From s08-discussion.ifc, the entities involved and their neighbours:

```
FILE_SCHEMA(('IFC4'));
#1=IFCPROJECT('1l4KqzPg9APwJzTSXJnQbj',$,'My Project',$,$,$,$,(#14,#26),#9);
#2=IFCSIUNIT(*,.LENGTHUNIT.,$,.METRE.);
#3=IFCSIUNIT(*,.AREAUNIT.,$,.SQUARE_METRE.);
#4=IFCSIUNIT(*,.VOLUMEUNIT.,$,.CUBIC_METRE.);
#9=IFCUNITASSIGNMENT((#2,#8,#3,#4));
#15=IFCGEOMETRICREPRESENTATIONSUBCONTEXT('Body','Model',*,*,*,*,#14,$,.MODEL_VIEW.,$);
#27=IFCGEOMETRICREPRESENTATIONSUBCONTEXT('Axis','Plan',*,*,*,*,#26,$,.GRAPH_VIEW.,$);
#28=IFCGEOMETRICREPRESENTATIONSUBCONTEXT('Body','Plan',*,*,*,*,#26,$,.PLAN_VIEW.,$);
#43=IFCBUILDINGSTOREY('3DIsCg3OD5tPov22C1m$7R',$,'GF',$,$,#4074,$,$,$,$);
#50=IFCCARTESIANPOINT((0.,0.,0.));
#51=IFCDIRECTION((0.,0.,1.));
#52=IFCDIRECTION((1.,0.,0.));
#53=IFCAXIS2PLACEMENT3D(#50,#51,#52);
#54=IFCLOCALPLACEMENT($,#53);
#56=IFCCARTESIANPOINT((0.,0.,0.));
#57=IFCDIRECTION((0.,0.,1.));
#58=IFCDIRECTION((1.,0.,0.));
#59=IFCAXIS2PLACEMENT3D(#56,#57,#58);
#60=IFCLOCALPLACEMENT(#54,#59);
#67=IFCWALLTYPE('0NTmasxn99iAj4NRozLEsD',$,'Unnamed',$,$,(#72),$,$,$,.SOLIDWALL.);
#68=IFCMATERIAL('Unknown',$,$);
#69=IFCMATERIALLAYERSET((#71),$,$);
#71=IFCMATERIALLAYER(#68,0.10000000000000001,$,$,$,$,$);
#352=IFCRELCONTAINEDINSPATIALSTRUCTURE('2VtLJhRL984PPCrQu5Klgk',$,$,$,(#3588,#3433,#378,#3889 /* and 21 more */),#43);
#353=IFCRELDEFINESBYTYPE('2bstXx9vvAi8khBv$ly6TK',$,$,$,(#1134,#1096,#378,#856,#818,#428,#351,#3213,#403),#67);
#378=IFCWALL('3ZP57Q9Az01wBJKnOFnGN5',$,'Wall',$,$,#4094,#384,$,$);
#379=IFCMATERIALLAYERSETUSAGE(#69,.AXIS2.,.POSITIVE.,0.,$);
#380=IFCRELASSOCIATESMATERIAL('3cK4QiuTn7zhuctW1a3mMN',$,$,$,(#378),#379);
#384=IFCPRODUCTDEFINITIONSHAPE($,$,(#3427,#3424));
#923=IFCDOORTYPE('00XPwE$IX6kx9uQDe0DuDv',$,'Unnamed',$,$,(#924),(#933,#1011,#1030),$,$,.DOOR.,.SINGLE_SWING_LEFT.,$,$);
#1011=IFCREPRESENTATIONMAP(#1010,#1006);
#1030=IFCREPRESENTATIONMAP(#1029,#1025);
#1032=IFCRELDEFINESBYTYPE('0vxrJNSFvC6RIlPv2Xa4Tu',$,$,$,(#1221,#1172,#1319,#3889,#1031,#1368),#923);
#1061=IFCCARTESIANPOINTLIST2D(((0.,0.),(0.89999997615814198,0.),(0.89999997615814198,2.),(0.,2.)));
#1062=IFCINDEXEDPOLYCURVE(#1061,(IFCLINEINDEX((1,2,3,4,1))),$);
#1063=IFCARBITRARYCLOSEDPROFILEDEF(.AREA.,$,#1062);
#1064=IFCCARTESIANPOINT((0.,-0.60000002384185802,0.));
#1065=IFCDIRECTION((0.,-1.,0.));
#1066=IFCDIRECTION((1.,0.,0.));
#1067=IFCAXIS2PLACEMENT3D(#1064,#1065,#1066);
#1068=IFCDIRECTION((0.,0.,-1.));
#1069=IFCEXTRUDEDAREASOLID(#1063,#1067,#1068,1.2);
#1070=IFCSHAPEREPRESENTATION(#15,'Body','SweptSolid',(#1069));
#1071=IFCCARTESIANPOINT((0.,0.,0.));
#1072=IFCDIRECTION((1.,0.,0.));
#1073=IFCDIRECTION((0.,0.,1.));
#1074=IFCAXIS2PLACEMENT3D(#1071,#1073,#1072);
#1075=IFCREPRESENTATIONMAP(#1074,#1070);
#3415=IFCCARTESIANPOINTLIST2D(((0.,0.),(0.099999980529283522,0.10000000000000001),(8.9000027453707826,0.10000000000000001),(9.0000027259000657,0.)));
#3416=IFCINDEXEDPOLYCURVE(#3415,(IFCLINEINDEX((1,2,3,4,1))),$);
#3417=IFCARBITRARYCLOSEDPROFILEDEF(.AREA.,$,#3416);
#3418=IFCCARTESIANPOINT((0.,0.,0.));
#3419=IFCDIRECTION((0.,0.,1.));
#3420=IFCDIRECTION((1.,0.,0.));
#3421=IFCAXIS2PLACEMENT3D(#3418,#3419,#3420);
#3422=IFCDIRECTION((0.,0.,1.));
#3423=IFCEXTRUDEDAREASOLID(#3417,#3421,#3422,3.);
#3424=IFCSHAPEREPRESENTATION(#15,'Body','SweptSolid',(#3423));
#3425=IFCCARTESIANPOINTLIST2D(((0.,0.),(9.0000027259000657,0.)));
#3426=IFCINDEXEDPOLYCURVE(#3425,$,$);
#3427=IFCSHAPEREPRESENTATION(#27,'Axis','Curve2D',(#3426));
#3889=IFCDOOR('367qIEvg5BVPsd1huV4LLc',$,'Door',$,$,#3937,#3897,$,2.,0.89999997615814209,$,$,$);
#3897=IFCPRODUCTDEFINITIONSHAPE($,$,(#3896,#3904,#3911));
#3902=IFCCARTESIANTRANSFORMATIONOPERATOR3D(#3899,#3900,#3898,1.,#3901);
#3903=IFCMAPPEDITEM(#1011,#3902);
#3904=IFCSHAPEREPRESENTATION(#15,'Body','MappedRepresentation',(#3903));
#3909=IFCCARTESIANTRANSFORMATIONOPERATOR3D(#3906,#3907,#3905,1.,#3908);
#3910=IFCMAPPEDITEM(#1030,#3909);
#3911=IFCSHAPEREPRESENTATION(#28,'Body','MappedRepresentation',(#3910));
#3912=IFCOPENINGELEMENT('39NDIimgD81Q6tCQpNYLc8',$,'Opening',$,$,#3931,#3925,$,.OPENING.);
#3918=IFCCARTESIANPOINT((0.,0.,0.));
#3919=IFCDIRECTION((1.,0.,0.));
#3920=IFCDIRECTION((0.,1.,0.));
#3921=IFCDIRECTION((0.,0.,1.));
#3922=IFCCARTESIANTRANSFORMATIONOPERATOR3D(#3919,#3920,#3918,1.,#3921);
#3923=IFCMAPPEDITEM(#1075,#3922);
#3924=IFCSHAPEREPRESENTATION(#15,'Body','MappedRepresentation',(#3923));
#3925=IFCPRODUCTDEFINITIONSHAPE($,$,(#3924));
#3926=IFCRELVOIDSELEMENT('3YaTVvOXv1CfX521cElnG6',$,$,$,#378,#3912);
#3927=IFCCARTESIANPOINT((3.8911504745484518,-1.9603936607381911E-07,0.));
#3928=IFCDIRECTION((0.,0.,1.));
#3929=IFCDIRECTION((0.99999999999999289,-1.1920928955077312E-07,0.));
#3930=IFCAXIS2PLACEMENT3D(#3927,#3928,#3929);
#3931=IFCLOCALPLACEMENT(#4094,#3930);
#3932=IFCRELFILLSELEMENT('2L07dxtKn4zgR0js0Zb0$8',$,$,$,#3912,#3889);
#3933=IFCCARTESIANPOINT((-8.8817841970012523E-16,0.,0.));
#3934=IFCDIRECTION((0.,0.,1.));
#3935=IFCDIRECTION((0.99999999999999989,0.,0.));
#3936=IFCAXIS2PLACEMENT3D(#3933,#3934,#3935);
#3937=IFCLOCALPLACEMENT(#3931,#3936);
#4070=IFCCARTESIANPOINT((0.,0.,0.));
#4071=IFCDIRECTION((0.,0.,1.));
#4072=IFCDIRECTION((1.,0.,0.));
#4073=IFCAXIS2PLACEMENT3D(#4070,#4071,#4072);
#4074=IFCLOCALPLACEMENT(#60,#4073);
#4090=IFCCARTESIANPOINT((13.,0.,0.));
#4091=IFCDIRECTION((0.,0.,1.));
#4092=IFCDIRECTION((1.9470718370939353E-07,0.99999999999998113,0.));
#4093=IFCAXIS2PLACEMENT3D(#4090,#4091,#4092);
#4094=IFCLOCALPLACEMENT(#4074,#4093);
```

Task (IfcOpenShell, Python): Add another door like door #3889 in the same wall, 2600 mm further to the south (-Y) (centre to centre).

```python
import ifcopenshell
import ifcopenshell.api.feature
import ifcopenshell.api.geometry
import ifcopenshell.api.root
import ifcopenshell.geom
import ifcopenshell.util.element
import ifcopenshell.util.placement
import ifcopenshell.util.shape
import ifcopenshell.util.unit

model = ifcopenshell.open("s08-discussion.ifc")
unit_scale = ifcopenshell.util.unit.calculate_unit_scale(model)
settings = ifcopenshell.geom.settings()


def volume(element):
    """Net volume in cubic metres, openings subtracted."""
    shape = ifcopenshell.geom.create_shape(settings, element)
    return ifcopenshell.util.shape.get_volume(shape.geometry)


door = model.by_guid("367qIEvg5BVPsd1huV4LLc")
opening = door.FillsVoids[0].RelatingOpeningElement
wall = opening.VoidsElements[0].RelatingBuildingElement
before = volume(wall)
shift = ifcopenshell.util.placement.get_local_placement(wall.ObjectPlacement)[:3, 0] * -2.6 / unit_scale

# copy_class copies the void relationship, type, container and properties, but no geometry.
new_opening = ifcopenshell.api.root.copy_class(model, product=opening)
new_opening.Representation = ifcopenshell.util.element.copy_deep(
    model, opening.Representation, exclude=["IfcGeometricRepresentationContext", "IfcRepresentationMap"]
)
new_door = ifcopenshell.api.root.copy_class(model, product=door)
new_door.Representation = ifcopenshell.util.element.copy_deep(
    model, door.Representation, exclude=["IfcGeometricRepresentationContext", "IfcRepresentationMap"]
)
ifcopenshell.api.feature.add_filling(model, opening=new_opening, element=new_door)

for old, new in ((opening, new_opening), (door, new_door)):
    matrix = ifcopenshell.util.placement.get_local_placement(old.ObjectPlacement)
    matrix[:3, 3] += shift
    ifcopenshell.api.geometry.edit_object_placement(model, product=new, matrix=matrix, is_si=False)

after = volume(wall)

print(f"wall volume {before:.3f} -> {after:.3f} m3")

model.write("s08-discussion_rev.ifc")
```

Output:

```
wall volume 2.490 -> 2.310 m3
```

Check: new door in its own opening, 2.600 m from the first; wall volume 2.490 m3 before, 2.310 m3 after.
